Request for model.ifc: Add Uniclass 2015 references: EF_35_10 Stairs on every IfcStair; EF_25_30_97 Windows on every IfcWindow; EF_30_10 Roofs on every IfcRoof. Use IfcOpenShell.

First a look at what the model holds.

```python
import ifcopenshell

model = ifcopenshell.open("model.ifc")
print(model.schema)
print("classifications:", [c.Name for c in model.by_type("IfcClassification")])
for ifc_class in ("IfcDoor", "IfcRoof", "IfcStair", "IfcWall", "IfcWindow"):
    print(ifc_class, len(model.by_type(ifc_class)))
```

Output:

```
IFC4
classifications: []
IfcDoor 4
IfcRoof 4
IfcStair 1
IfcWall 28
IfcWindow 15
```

```python
import ifcopenshell
import ifcopenshell.api.classification

model = ifcopenshell.open("model.ifc")

system = ifcopenshell.api.classification.add_classification(model, classification="Uniclass 2015")

codes = {
    "IfcStair": ("EF_35_10", "Stairs"),
    "IfcWindow": ("EF_25_30_97", "Windows"),
    "IfcRoof": ("EF_30_10", "Roofs"),
}
for ifc_class, (code, name) in codes.items():
    products = model.by_type(ifc_class)
    ifcopenshell.api.classification.add_reference(
        model, products=products, classification=system, identification=code, name=name
    )
    print(code, len(products))

model.write("model_v2.ifc")
```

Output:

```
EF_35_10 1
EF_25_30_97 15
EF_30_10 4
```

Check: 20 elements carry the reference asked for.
